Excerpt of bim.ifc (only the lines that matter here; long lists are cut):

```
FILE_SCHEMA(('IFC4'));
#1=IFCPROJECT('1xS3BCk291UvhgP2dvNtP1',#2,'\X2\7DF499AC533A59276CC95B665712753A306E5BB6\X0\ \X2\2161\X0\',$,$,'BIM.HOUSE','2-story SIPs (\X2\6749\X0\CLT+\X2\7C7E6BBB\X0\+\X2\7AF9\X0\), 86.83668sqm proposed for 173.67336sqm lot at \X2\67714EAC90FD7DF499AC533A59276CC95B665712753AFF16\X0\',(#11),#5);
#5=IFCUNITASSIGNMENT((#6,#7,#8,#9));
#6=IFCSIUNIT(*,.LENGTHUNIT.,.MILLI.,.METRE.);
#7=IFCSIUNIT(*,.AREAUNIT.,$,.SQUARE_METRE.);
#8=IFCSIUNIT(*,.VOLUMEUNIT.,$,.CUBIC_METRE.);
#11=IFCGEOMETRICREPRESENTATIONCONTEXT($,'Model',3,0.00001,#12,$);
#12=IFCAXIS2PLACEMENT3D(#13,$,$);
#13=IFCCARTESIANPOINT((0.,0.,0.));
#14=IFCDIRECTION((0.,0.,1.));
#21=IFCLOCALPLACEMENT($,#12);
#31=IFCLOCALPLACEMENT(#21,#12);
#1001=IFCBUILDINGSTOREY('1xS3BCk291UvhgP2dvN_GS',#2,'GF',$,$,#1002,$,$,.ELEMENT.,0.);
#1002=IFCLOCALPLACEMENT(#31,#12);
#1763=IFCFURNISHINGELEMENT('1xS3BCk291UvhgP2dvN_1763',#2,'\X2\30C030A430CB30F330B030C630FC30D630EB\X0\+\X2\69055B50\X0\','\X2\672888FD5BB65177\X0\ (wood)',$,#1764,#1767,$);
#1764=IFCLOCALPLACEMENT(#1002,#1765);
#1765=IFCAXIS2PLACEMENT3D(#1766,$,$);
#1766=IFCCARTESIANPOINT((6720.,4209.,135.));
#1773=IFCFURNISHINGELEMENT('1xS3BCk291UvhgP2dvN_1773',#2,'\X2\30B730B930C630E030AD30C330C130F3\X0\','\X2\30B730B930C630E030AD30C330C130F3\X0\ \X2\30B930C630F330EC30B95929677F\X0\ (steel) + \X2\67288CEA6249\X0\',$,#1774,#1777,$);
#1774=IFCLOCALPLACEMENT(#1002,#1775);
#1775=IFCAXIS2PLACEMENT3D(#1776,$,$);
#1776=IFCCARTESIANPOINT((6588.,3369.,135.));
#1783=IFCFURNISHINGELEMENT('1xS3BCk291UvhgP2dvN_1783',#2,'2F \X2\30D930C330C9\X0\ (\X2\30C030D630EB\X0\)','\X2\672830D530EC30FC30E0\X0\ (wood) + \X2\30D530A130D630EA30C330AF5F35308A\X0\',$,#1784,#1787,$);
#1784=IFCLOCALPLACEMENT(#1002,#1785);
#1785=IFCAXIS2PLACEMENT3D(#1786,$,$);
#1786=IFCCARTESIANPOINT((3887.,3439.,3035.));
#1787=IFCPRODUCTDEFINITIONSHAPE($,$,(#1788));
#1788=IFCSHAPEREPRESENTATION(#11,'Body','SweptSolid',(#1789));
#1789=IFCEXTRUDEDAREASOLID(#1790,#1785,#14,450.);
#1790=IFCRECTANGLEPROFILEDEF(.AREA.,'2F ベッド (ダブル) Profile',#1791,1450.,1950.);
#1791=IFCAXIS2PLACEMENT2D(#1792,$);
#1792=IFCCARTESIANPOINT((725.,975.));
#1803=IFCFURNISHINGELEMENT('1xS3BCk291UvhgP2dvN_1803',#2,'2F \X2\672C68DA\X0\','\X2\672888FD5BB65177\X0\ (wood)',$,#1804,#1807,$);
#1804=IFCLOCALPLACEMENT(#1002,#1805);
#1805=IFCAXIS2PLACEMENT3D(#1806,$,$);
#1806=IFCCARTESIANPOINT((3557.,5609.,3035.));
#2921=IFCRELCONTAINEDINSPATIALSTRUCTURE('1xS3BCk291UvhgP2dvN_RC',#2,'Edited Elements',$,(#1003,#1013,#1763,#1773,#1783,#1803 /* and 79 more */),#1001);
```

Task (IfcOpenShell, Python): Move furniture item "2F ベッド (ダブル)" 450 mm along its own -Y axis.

```python
import ifcopenshell
import ifcopenshell.api.geometry
import ifcopenshell.util.placement

model = ifcopenshell.open("bim.ifc")

item = model.by_guid("1xS3BCk291UvhgP2dvN_1783")
matrix = ifcopenshell.util.placement.get_local_placement(item.ObjectPlacement)
matrix[:3, 3] -= matrix[:3, 1] * 450.0
ifcopenshell.api.geometry.edit_object_placement(model, product=item, matrix=matrix, is_si=False)

print(ifcopenshell.util.placement.get_local_placement(item.ObjectPlacement).round(3) + 0.0)

model.write("bim_updated.ifc")
```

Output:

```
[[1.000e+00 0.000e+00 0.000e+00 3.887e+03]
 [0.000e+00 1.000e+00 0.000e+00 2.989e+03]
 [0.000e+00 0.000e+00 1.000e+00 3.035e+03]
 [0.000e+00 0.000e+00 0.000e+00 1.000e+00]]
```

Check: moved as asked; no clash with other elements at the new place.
